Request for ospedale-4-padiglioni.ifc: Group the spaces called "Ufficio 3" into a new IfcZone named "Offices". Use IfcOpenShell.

First a look at what the model holds.

```python
import ifcopenshell

model = ifcopenshell.open("ospedale-4-padiglioni.ifc")
print(model.schema)
seen = {}
for space in model.by_type("IfcSpace"):
    seen[space.LongName] = seen.get(space.LongName, 0) + 1
for name, count in sorted(seen.items(), key=str):
    print(count, "x", name)
print("zones:", [z.Name for z in model.by_type("IfcZone")][:20])
```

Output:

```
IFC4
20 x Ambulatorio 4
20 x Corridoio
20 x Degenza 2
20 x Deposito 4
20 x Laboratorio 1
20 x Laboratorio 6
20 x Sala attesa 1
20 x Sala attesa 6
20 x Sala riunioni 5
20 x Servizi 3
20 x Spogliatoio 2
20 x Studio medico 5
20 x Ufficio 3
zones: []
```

```python
import ifcopenshell
import ifcopenshell.api.group
import ifcopenshell.api.root

model = ifcopenshell.open("ospedale-4-padiglioni.ifc")

names = {"Ufficio 3"}
spaces = [s for s in model.by_type("IfcSpace") if s.LongName in names]

zone = ifcopenshell.api.root.create_entity(model, ifc_class="IfcZone", name="Offices")
ifcopenshell.api.group.assign_group(model, products=spaces, group=zone)
print(len(spaces), "spaces in", zone.Name)

model.write("ospedale-4-padiglioni_rev.ifc")
```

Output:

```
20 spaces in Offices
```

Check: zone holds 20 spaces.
